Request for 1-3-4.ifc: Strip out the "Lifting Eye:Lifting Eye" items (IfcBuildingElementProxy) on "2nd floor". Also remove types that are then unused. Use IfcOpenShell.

First a look at what the model holds.

```python
import ifcopenshell
import ifcopenshell.util.element

model = ifcopenshell.open("1-3-4.ifc")
print(model.schema)
storey = next(s for s in model.by_type("IfcBuildingStorey") if s.Name == "2nd floor")
proxies = [e for e in ifcopenshell.util.element.get_decomposition(storey) if e.is_a("IfcBuildingElementProxy")]
seen = {}
for e in proxies:
    element_type = ifcopenshell.util.element.get_type(e)
    name = element_type.Name if element_type not in (None, e) else None
    seen[name] = seen.get(name, 0) + 1
for name, count in sorted(seen.items(), key=str):
    print(count, "x", name)
```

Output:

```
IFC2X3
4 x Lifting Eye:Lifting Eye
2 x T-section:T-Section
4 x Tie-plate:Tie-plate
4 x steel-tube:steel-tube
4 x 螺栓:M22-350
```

```python
import ifcopenshell
import ifcopenshell.api.root
import ifcopenshell.util.element

model = ifcopenshell.open("1-3-4.ifc")

storey = next(s for s in model.by_type("IfcBuildingStorey") if s.Name == "2nd floor")
proxies = [e for e in ifcopenshell.util.element.get_decomposition(storey) if e.is_a("IfcBuildingElementProxy")]
targets = [e for e in proxies if (t := ifcopenshell.util.element.get_type(e)) not in (None, e) and t.Name == "Lifting Eye:Lifting Eye"]
types = {ifcopenshell.util.element.get_type(e) for e in targets} - {None, *targets}

for e in targets:
    ifcopenshell.api.root.remove_product(model, product=e)
print(len(targets), "removed")

unused = [t for t in types if not ifcopenshell.util.element.get_types(t)]
for t in unused:
    ifcopenshell.api.root.remove_product(model, product=t)
print(len(unused), "unused types removed")

model.write("1-3-4_updated.ifc")
```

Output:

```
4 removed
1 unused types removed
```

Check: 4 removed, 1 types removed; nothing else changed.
